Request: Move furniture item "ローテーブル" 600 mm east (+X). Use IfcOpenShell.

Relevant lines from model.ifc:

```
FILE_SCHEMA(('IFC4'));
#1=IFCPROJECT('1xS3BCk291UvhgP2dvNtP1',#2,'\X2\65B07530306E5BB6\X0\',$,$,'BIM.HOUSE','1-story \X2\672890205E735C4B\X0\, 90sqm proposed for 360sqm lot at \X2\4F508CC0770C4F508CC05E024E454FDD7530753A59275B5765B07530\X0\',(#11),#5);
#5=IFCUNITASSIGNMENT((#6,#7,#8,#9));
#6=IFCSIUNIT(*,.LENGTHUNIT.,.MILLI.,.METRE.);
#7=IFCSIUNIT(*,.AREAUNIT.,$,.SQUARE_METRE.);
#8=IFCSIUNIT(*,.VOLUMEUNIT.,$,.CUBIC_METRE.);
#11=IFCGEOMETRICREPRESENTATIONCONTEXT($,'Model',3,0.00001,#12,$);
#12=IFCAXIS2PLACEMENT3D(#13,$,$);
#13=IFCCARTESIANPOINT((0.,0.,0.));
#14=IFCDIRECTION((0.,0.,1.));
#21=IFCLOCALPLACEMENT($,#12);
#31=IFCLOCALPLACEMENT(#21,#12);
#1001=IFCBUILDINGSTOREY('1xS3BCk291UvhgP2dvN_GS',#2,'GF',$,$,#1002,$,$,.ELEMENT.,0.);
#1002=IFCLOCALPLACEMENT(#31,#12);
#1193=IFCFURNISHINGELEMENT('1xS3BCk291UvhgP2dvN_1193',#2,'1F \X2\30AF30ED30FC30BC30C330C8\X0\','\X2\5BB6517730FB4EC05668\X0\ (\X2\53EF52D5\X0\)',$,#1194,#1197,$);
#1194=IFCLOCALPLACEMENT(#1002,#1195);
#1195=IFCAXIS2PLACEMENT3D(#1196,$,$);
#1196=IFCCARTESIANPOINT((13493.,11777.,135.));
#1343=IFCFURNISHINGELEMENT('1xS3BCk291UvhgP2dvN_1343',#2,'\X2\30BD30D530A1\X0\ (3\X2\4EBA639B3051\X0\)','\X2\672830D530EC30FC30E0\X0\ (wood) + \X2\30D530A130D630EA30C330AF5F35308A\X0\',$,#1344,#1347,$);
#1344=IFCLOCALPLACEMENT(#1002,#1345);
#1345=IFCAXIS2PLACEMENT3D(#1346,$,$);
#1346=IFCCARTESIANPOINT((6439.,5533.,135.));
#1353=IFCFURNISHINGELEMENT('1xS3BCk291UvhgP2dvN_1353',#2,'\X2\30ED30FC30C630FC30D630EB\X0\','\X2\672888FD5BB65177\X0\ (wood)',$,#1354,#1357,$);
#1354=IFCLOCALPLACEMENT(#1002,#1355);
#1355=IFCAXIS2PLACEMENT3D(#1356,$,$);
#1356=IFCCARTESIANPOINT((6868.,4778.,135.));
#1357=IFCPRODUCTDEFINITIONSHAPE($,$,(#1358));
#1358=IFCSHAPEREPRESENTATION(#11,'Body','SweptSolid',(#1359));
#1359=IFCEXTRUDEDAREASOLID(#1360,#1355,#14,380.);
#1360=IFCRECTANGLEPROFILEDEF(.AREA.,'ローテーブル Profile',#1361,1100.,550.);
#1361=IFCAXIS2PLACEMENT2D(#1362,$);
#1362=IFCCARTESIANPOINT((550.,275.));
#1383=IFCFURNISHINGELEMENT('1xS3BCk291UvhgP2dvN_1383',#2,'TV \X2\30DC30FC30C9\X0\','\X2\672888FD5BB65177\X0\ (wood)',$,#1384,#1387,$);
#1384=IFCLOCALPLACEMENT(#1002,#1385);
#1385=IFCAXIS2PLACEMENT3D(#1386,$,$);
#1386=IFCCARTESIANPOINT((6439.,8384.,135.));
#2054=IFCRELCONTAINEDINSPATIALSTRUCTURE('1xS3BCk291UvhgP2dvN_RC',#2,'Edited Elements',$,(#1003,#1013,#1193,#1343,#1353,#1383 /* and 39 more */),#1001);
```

```python
import ifcopenshell
import ifcopenshell.api.geometry
import ifcopenshell.util.placement
import ifcopenshell.util.unit

model = ifcopenshell.open("model.ifc")
unit_scale = ifcopenshell.util.unit.calculate_unit_scale(model)

item = model.by_guid("1xS3BCk291UvhgP2dvN_1353")
matrix = ifcopenshell.util.placement.get_local_placement(item.ObjectPlacement)
matrix[0, 3] += 0.6 / unit_scale
ifcopenshell.api.geometry.edit_object_placement(model, product=item, matrix=matrix, is_si=False)

print(ifcopenshell.util.placement.get_local_placement(item.ObjectPlacement).round(3) + 0.0)

model.write("model-out.ifc")
```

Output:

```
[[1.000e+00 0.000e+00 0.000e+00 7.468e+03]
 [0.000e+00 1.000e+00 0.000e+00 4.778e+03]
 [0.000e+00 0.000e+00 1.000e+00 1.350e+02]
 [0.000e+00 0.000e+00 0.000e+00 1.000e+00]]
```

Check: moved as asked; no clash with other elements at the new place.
